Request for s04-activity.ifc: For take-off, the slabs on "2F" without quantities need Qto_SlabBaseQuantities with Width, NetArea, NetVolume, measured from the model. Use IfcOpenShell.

First a look at what the model holds.

```python
import ifcopenshell
import ifcopenshell.util.element
import ifcopenshell.util.unit

model = ifcopenshell.open("s04-activity.ifc")
print(model.schema)
for unit_type in ("LENGTHUNIT", "AREAUNIT", "VOLUMEUNIT"):
    print(unit_type, ifcopenshell.util.unit.calculate_unit_scale(model, unit_type))
storey = next(s for s in model.by_type("IfcBuildingStorey") if s.Name == "2F")
slabs = [e for e in ifcopenshell.util.element.get_decomposition(storey) if e.is_a("IfcSlab")]
for e in sorted(slabs, key=lambda e: e.id()):
    print(e.id(), e.is_a(), e.Name, list(ifcopenshell.util.element.get_psets(e, qtos_only=True)), sep=" | ")
```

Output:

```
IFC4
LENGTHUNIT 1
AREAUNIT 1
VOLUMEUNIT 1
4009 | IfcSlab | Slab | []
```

```python
import ifcopenshell
import ifcopenshell.api.pset
import ifcopenshell.geom
import ifcopenshell.util.element
import ifcopenshell.util.shape
import ifcopenshell.util.unit

model = ifcopenshell.open("s04-activity.ifc")
unit_scale = ifcopenshell.util.unit.calculate_unit_scale(model)
area_scale = ifcopenshell.util.unit.calculate_unit_scale(model, "AREAUNIT")
volume_scale = ifcopenshell.util.unit.calculate_unit_scale(model, "VOLUMEUNIT")
settings = ifcopenshell.geom.settings()

storey = next(s for s in model.by_type("IfcBuildingStorey") if s.Name == "2F")
slabs = [e for e in ifcopenshell.util.element.get_decomposition(storey) if e.is_a("IfcSlab")]

for e in sorted(slabs, key=lambda e: e.id()):
    if ifcopenshell.util.element.get_psets(e, qtos_only=True, should_inherit=False):
        continue
    # Geometry comes back in metres, in the element's own axes.
    shape = ifcopenshell.geom.create_shape(settings, e)
    values = {
        "Width": ifcopenshell.util.shape.get_z(shape.geometry) / unit_scale,
        "NetArea": ifcopenshell.util.shape.get_footprint_area(shape.geometry) / area_scale,
        "NetVolume": ifcopenshell.util.shape.get_volume(shape.geometry) / volume_scale,
    }
    qto = ifcopenshell.api.pset.add_qto(model, product=e, name="Qto_SlabBaseQuantities")
    ifcopenshell.api.pset.edit_qto(model, qto=qto, properties=values)
    print(e.id(), {k: round(v, 3) for k, v in values.items()})

model.write("s04-activity_edited.ifc")
```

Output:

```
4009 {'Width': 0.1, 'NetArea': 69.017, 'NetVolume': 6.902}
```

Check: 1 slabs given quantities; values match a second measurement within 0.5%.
